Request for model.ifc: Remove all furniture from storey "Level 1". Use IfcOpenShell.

First a look at what the model holds.

```python
import ifcopenshell
import ifcopenshell.util.element

model = ifcopenshell.open("model.ifc")
print(model.schema)
storey = next(s for s in model.by_type("IfcBuildingStorey") if s.Name == "Level 1")
furniture = [e for e in ifcopenshell.util.element.get_decomposition(storey) if e.is_a("IfcFurnishingElement")]
seen = {}
for e in furniture:
    element_type = ifcopenshell.util.element.get_type(e)
    name = element_type.Name if element_type not in (None, e) else None
    seen[name] = seen.get(name, 0) + 1
for name, count in sorted(seen.items(), key=str):
    print(count, "x", name)
```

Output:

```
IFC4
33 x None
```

```python
import ifcopenshell
import ifcopenshell.api.root
import ifcopenshell.util.element

model = ifcopenshell.open("model.ifc")

storey = next(s for s in model.by_type("IfcBuildingStorey") if s.Name == "Level 1")
furniture = [e for e in ifcopenshell.util.element.get_decomposition(storey) if e.is_a("IfcFurnishingElement")]

for e in furniture:
    ifcopenshell.api.root.remove_product(model, product=e)
print(len(furniture), "removed")

model.write("model_updated.ifc")
```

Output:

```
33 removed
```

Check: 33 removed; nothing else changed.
